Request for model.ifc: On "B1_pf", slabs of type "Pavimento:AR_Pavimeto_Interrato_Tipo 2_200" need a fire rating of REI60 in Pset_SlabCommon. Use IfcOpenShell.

First a look at what the model holds.

```python
import ifcopenshell
import ifcopenshell.util.element

model = ifcopenshell.open("model.ifc")
print(model.schema)
storey = next(s for s in model.by_type("IfcBuildingStorey") if s.Name == "B1_pf")
slabs = [e for e in ifcopenshell.util.element.get_decomposition(storey) if e.is_a("IfcSlab")]
seen = {}
for e in slabs:
    element_type = ifcopenshell.util.element.get_type(e)
    key = (element_type.Name if element_type != e and element_type else None, ifcopenshell.util.element.get_pset(e, "Pset_SlabCommon", "FireRating"))
    seen[key] = seen.get(key, 0) + 1
for (name, value), count in sorted(seen.items(), key=str):
    print(count, "x", name, "|", value)
```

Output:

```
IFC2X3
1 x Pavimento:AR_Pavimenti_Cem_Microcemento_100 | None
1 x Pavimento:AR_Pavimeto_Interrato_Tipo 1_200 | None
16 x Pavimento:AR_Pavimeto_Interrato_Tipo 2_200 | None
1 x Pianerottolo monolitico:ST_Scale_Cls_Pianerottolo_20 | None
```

```python
import ifcopenshell
import ifcopenshell.api.pset
import ifcopenshell.util.element

model = ifcopenshell.open("model.ifc")

storey = next(s for s in model.by_type("IfcBuildingStorey") if s.Name == "B1_pf")
slabs = [e for e in ifcopenshell.util.element.get_decomposition(storey) if e.is_a("IfcSlab")]

count = 0
for e in slabs:
    element_type = ifcopenshell.util.element.get_type(e)
    if element_type in (None, e) or element_type.Name != "Pavimento:AR_Pavimeto_Interrato_Tipo 2_200":
        continue
    # add_pset returns the element's existing set when there is one.
    pset = ifcopenshell.api.pset.add_pset(model, product=e, name="Pset_SlabCommon")
    ifcopenshell.api.pset.edit_pset(model, pset=pset, properties={"FireRating": "REI60"})
    count += 1

print(count, "slabs updated")

model.write("model_rev.ifc")
```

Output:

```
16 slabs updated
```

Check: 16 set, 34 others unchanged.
